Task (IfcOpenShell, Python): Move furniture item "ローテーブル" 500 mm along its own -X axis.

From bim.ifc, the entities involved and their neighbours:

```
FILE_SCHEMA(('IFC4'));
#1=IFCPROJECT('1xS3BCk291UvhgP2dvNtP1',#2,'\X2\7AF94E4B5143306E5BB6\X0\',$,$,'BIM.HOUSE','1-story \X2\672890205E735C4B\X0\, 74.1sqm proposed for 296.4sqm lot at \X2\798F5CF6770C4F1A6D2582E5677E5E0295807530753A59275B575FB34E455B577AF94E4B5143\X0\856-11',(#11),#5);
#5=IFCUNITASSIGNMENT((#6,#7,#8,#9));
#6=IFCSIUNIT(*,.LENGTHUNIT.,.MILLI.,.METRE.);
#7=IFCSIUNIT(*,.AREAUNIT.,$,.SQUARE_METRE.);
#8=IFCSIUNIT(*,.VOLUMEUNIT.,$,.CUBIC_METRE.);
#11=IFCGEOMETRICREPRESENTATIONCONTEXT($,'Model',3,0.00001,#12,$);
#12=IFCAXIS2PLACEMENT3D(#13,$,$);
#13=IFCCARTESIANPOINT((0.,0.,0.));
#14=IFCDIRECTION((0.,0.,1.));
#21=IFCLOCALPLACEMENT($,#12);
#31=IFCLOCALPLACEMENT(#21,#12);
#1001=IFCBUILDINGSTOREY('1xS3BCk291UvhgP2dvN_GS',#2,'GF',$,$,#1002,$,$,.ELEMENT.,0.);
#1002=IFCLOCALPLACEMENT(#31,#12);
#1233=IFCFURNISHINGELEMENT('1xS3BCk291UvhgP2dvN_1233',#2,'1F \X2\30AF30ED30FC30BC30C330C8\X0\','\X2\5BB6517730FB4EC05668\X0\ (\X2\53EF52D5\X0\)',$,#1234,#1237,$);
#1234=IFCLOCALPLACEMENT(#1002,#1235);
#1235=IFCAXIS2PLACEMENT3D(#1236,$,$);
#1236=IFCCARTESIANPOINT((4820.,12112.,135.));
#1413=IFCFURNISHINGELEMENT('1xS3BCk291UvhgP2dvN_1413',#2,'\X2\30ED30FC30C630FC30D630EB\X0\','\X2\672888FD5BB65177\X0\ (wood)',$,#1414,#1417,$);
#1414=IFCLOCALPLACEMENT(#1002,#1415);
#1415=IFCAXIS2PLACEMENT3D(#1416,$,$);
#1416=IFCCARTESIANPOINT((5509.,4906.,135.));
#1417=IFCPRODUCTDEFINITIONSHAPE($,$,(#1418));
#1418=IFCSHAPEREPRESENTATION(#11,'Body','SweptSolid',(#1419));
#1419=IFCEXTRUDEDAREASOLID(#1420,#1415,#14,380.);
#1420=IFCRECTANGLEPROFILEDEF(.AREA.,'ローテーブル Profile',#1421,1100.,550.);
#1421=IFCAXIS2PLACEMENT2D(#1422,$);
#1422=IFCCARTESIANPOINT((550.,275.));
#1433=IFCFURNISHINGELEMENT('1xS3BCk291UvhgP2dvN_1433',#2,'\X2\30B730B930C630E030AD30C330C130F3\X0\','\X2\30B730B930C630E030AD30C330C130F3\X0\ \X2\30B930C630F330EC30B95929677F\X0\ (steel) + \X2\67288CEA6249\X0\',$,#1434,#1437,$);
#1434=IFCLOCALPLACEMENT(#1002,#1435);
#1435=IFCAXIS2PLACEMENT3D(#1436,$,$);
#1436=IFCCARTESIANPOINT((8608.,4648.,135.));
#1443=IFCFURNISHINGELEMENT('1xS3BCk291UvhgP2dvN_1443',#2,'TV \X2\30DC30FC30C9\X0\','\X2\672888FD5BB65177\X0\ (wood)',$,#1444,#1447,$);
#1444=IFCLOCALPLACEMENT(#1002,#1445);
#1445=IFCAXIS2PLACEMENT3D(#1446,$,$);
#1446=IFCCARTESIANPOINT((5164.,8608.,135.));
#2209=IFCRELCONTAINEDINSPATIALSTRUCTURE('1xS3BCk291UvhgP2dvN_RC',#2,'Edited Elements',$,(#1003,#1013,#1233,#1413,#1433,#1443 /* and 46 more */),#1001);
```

```python
import ifcopenshell
import ifcopenshell.api.geometry
import ifcopenshell.util.placement

model = ifcopenshell.open("bim.ifc")

item = model.by_guid("1xS3BCk291UvhgP2dvN_1413")
matrix = ifcopenshell.util.placement.get_local_placement(item.ObjectPlacement)
matrix[:3, 3] -= matrix[:3, 0] * 500.0
ifcopenshell.api.geometry.edit_object_placement(model, product=item, matrix=matrix, is_si=False)

print(ifcopenshell.util.placement.get_local_placement(item.ObjectPlacement).round(3) + 0.0)

model.write("bim_updated.ifc")
```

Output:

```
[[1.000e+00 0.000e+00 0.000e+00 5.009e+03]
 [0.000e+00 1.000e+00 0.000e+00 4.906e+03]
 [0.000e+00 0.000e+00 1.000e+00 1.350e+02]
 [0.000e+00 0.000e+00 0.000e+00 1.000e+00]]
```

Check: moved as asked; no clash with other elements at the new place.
